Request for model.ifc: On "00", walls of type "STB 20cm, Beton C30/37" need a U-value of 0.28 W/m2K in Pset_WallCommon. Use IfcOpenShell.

First a look at what the model holds.

```python
import ifcopenshell
import ifcopenshell.util.element

model = ifcopenshell.open("model.ifc")
print(model.schema)
storey = next(s for s in model.by_type("IfcBuildingStorey") if s.Name == "00")
walls = [e for e in ifcopenshell.util.element.get_decomposition(storey) if e.is_a("IfcWall")]
seen = {}
for e in walls:
    element_type = ifcopenshell.util.element.get_type(e)
    key = (element_type.Name if element_type != e and element_type else None, ifcopenshell.util.element.get_pset(e, "Pset_WallCommon", "ThermalTransmittance"))
    seen[key] = seen.get(key, 0) + 1
for (name, value), count in sorted(seen.items(), key=str):
    print(count, "x", name, "|", value)
```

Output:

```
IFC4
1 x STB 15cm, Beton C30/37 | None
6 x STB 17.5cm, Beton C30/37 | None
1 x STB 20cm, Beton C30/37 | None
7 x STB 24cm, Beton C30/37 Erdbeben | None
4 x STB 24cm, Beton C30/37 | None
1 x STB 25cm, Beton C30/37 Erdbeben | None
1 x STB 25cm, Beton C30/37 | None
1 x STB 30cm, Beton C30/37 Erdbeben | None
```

```python
import ifcopenshell
import ifcopenshell.api.pset
import ifcopenshell.util.element

model = ifcopenshell.open("model.ifc")

storey = next(s for s in model.by_type("IfcBuildingStorey") if s.Name == "00")
walls = [e for e in ifcopenshell.util.element.get_decomposition(storey) if e.is_a("IfcWall")]

count = 0
for e in walls:
    element_type = ifcopenshell.util.element.get_type(e)
    if element_type in (None, e) or element_type.Name != "STB 20cm, Beton C30/37":
        continue
    # add_pset returns the element's existing set when there is one.
    pset = ifcopenshell.api.pset.add_pset(model, product=e, name="Pset_WallCommon")
    ifcopenshell.api.pset.edit_pset(model, pset=pset, properties={"ThermalTransmittance": 0.28})
    count += 1

print(count, "walls updated")

model.write("model-out.ifc")
```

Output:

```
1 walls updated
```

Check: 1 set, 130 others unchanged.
